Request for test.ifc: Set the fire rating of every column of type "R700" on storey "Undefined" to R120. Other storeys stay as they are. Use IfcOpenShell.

First a look at what the model holds.

```python
import ifcopenshell
import ifcopenshell.util.element

model = ifcopenshell.open("test.ifc")
print(model.schema)
storey = next(s for s in model.by_type("IfcBuildingStorey") if s.Name == "Undefined")
columns = [e for e in ifcopenshell.util.element.get_decomposition(storey) if e.is_a("IfcColumn")]
seen = {}
for e in columns:
    element_type = ifcopenshell.util.element.get_type(e)
    key = (element_type.Name if element_type != e and element_type else None, ifcopenshell.util.element.get_pset(e, "Pset_ColumnCommon", "FireRating"))
    seen[key] = seen.get(key, 0) + 1
for (name, value), count in sorted(seen.items(), key=str):
    print(count, "x", name, "|", value)
```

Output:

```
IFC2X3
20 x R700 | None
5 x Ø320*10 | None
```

```python
import ifcopenshell
import ifcopenshell.api.pset
import ifcopenshell.util.element

model = ifcopenshell.open("test.ifc")

storey = next(s for s in model.by_type("IfcBuildingStorey") if s.Name == "Undefined")
columns = [e for e in ifcopenshell.util.element.get_decomposition(storey) if e.is_a("IfcColumn")]

count = 0
for e in columns:
    element_type = ifcopenshell.util.element.get_type(e)
    if element_type in (None, e) or element_type.Name != "R700":
        continue
    found = ifcopenshell.util.element.get_pset(e, "Pset_ColumnCommon", should_inherit=False)
    if found:
        pset = model.by_id(found["id"])
        if len(ifcopenshell.util.element.get_elements_by_pset(pset)) > 1:
            pset = ifcopenshell.api.pset.unshare_pset(model, products=[e], pset=pset)[0]
    else:
        pset = ifcopenshell.api.pset.add_pset(model, product=e, name="Pset_ColumnCommon")
    ifcopenshell.api.pset.edit_pset(model, pset=pset, properties={"FireRating": "R120"})
    count += 1

print(count, "columns updated")

model.write("test_updated.ifc")
```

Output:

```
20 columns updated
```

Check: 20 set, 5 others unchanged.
